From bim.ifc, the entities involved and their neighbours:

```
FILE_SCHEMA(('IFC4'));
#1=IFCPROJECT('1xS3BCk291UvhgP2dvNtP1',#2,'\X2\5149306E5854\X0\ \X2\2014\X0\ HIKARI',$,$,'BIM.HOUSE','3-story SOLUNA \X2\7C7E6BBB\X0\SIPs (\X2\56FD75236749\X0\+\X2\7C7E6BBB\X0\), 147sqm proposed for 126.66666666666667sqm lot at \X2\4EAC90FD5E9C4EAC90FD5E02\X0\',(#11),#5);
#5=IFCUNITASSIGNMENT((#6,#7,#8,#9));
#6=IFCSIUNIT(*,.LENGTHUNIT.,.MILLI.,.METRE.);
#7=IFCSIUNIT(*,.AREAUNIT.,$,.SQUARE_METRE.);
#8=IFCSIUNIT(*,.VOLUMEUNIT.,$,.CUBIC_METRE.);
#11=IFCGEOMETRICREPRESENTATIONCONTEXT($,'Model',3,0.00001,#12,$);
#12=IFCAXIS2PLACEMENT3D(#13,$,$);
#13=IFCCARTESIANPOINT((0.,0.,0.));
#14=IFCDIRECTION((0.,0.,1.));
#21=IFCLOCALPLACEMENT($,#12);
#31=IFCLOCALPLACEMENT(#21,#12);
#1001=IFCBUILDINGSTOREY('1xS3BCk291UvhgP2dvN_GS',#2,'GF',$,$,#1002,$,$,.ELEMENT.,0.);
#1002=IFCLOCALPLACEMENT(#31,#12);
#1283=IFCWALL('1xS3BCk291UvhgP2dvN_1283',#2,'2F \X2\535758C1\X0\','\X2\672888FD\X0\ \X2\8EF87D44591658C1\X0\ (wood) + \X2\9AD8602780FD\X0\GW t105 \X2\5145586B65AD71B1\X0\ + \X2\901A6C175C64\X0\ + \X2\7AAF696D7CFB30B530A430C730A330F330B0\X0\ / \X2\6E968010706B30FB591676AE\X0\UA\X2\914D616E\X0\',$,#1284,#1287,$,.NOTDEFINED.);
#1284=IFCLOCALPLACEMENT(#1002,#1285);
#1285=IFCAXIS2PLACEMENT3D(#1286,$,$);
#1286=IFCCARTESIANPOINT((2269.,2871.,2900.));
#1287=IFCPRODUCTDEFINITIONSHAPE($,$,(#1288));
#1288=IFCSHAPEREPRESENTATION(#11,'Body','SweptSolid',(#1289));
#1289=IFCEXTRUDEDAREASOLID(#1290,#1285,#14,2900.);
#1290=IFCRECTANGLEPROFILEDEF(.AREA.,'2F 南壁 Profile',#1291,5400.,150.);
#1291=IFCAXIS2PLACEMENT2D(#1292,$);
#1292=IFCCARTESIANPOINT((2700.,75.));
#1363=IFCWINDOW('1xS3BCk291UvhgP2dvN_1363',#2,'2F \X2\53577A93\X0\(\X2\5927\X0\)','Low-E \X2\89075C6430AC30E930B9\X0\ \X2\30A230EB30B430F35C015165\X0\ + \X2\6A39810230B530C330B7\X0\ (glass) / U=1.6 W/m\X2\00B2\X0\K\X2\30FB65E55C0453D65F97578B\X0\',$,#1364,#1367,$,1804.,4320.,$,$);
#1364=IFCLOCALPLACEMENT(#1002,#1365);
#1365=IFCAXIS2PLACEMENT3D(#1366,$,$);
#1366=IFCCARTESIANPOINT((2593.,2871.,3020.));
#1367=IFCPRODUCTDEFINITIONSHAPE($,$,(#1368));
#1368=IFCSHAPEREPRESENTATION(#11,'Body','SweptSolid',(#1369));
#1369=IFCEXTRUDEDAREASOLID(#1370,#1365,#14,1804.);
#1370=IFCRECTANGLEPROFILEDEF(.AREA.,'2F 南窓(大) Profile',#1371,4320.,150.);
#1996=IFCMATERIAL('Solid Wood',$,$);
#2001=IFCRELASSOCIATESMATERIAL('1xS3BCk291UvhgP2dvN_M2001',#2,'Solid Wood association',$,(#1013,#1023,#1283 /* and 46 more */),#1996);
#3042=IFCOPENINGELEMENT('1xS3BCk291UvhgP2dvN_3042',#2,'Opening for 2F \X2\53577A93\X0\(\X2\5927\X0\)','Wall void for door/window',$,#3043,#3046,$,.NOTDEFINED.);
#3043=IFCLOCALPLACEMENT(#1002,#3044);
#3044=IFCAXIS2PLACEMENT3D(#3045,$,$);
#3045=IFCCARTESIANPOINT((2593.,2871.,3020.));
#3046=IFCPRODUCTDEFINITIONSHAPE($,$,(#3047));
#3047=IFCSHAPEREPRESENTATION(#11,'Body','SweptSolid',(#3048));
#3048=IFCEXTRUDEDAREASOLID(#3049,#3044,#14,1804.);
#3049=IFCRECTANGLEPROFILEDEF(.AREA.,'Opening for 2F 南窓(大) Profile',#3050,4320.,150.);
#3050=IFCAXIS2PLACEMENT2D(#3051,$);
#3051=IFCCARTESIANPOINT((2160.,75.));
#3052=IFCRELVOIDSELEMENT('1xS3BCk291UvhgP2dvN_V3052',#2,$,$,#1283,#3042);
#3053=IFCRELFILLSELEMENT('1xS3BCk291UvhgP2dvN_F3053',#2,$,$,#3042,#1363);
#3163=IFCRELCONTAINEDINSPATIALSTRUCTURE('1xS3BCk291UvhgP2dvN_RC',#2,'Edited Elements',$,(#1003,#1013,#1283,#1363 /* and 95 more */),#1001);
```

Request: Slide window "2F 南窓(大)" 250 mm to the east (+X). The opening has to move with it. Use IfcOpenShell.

```python
import ifcopenshell
import ifcopenshell.api.geometry
import ifcopenshell.util.placement
import ifcopenshell.util.unit

model = ifcopenshell.open("bim.ifc")
unit_scale = ifcopenshell.util.unit.calculate_unit_scale(model)

window = model.by_id(1363)
opening = window.FillsVoids[0].RelatingOpeningElement
wall = opening.VoidsElements[0].RelatingBuildingElement

wall_matrix = ifcopenshell.util.placement.get_local_placement(wall.ObjectPlacement)
shift = wall_matrix[:3, 0] * 0.25 / unit_scale
before = ifcopenshell.util.placement.get_local_placement(window.ObjectPlacement)[:3, 3].copy()

# The window is not placed relative to its opening, so move both.
for product in (opening, window):
    matrix = ifcopenshell.util.placement.get_local_placement(product.ObjectPlacement)
    matrix[:3, 3] += shift
    ifcopenshell.api.geometry.edit_object_placement(model, product=product, matrix=matrix, is_si=False)

after = ifcopenshell.util.placement.get_local_placement(window.ObjectPlacement)[:3, 3]
print("window moved by", (after - before).round(3) + 0.0)

model.write("bim_rev.ifc")
```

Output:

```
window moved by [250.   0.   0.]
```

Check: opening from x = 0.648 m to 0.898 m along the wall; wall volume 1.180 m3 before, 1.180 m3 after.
